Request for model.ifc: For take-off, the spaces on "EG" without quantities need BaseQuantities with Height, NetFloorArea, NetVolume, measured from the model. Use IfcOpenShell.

First a look at what the model holds.

```python
import ifcopenshell
import ifcopenshell.util.element
import ifcopenshell.util.unit

model = ifcopenshell.open("model.ifc")
print(model.schema)
for unit_type in ("LENGTHUNIT", "AREAUNIT", "VOLUMEUNIT"):
    print(unit_type, ifcopenshell.util.unit.calculate_unit_scale(model, unit_type))
storey = next(s for s in model.by_type("IfcBuildingStorey") if s.Name == "EG")
spaces = [e for e in ifcopenshell.util.element.get_decomposition(storey) if e.is_a("IfcSpace")]
for e in sorted(spaces, key=lambda e: e.id()):
    print(e.id(), e.is_a(), e.Name, list(ifcopenshell.util.element.get_psets(e, qtos_only=True)), sep=" | ")
```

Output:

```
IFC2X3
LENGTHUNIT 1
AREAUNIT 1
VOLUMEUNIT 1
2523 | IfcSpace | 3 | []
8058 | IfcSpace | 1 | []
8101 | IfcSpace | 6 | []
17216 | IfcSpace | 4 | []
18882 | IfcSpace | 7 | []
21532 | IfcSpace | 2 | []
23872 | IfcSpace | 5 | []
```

```python
import ifcopenshell
import ifcopenshell.api.pset
import ifcopenshell.geom
import ifcopenshell.util.element
import ifcopenshell.util.shape
import ifcopenshell.util.unit

model = ifcopenshell.open("model.ifc")
unit_scale = ifcopenshell.util.unit.calculate_unit_scale(model)
area_scale = ifcopenshell.util.unit.calculate_unit_scale(model, "AREAUNIT")
volume_scale = ifcopenshell.util.unit.calculate_unit_scale(model, "VOLUMEUNIT")
settings = ifcopenshell.geom.settings()

storey = next(s for s in model.by_type("IfcBuildingStorey") if s.Name == "EG")
spaces = [e for e in ifcopenshell.util.element.get_decomposition(storey) if e.is_a("IfcSpace")]

for e in sorted(spaces, key=lambda e: e.id()):
    if ifcopenshell.util.element.get_psets(e, qtos_only=True, should_inherit=False):
        continue
    # Geometry comes back in metres, in the element's own axes.
    shape = ifcopenshell.geom.create_shape(settings, e)
    values = {
        "Height": ifcopenshell.util.shape.get_z(shape.geometry) / unit_scale,
        "NetFloorArea": ifcopenshell.util.shape.get_footprint_area(shape.geometry) / area_scale,
        "NetVolume": ifcopenshell.util.shape.get_volume(shape.geometry) / volume_scale,
    }
    qto = ifcopenshell.api.pset.add_qto(model, product=e, name="BaseQuantities")
    ifcopenshell.api.pset.edit_qto(model, qto=qto, properties=values)
    print(e.id(), {k: round(v, 3) for k, v in values.items()})

model.write("model_v2.ifc")
```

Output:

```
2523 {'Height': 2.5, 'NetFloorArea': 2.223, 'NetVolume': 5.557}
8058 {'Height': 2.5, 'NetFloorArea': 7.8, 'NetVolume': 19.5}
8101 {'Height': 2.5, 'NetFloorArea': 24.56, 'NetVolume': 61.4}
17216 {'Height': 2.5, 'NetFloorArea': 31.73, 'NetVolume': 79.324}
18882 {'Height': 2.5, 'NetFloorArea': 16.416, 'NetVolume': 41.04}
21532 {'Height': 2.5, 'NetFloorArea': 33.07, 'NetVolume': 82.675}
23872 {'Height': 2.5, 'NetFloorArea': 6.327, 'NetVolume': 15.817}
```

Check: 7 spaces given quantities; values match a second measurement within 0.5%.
